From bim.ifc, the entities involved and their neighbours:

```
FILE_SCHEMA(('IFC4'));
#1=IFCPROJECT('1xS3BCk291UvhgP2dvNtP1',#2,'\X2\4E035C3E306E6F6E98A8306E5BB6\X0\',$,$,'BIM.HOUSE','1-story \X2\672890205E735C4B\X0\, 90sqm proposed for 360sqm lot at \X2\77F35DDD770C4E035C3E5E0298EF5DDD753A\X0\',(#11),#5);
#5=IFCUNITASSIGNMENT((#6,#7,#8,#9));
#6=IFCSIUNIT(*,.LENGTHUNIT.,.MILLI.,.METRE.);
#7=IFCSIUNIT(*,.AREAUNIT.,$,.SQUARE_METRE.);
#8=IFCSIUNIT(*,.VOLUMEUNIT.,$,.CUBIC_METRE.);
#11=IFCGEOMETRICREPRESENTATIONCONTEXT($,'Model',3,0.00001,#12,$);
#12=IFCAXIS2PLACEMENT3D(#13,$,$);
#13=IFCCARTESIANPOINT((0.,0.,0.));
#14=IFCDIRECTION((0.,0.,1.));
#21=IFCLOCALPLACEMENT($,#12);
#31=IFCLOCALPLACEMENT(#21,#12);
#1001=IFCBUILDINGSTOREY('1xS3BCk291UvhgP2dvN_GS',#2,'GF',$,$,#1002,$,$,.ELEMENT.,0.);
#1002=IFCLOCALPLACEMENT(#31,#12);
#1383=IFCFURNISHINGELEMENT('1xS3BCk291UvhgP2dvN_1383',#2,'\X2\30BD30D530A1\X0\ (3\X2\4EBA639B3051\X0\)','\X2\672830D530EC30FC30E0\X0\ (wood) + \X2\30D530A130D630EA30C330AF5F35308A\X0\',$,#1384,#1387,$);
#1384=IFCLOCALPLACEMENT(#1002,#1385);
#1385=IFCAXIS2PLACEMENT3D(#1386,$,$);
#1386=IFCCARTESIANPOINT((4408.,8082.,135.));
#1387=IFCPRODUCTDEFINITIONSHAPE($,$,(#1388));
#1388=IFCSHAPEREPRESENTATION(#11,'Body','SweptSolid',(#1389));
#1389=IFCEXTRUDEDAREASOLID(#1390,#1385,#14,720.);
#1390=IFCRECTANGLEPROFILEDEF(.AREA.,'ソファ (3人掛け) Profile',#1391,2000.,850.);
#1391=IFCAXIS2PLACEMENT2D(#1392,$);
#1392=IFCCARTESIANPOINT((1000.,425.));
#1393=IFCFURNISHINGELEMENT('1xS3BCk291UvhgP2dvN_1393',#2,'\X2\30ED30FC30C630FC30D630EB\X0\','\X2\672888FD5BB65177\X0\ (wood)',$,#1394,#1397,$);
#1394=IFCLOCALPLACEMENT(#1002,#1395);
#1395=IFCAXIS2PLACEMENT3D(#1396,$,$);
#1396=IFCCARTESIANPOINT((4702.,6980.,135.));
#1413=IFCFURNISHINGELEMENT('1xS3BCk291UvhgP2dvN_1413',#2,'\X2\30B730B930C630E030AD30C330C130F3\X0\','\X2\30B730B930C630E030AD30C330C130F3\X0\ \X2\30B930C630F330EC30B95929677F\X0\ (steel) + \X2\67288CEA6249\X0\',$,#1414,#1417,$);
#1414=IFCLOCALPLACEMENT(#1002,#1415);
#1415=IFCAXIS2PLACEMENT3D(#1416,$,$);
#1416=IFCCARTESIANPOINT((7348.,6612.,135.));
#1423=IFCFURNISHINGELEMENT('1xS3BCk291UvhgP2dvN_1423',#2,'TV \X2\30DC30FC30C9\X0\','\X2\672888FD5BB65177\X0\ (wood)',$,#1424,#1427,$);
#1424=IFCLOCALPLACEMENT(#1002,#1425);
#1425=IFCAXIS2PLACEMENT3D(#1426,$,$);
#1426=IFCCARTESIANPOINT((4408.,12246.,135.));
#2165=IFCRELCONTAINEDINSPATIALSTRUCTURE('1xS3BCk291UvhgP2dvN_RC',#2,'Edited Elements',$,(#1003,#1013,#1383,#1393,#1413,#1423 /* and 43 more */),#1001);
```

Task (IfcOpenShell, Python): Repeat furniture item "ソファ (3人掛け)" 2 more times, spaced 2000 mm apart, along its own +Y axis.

```python
import ifcopenshell
import ifcopenshell.api.geometry
import ifcopenshell.api.root
import ifcopenshell.util.element
import ifcopenshell.util.placement
import ifcopenshell.util.unit

model = ifcopenshell.open("bim.ifc")
unit_scale = ifcopenshell.util.unit.calculate_unit_scale(model)


def reuse_history(source, copy):
    """copy_class also copies each property set's owner history, people and application; keep the originals."""
    for rel in copy.IsDefinedBy:
        if rel.is_a("IfcRelDefinesByProperties") and (history := rel.RelatingPropertyDefinition.OwnerHistory):
            rel.RelatingPropertyDefinition.OwnerHistory = source.OwnerHistory
            ifcopenshell.util.element.remove_deep2(model, history)


source = model.by_guid("1xS3BCk291UvhgP2dvN_1383")
base = ifcopenshell.util.placement.get_local_placement(source.ObjectPlacement)
step = base[:3, 1] * 2 / unit_scale

for i in range(1, 3):
    copy = ifcopenshell.api.root.copy_class(model, product=source)
    copy.Representation = ifcopenshell.util.element.copy_deep(
        model, source.Representation, exclude=["IfcGeometricRepresentationContext", "IfcRepresentationMap"]
    )
    reuse_history(source, copy)
    matrix = base.copy()
    matrix[:3, 3] += i * step
    print("added at", matrix[:3, 3].round(3) + 0.0)
    ifcopenshell.api.geometry.edit_object_placement(model, product=copy, matrix=matrix, is_si=False)

model.write("bim_edited.ifc")
```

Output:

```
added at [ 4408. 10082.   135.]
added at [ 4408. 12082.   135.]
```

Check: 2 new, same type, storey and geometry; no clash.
